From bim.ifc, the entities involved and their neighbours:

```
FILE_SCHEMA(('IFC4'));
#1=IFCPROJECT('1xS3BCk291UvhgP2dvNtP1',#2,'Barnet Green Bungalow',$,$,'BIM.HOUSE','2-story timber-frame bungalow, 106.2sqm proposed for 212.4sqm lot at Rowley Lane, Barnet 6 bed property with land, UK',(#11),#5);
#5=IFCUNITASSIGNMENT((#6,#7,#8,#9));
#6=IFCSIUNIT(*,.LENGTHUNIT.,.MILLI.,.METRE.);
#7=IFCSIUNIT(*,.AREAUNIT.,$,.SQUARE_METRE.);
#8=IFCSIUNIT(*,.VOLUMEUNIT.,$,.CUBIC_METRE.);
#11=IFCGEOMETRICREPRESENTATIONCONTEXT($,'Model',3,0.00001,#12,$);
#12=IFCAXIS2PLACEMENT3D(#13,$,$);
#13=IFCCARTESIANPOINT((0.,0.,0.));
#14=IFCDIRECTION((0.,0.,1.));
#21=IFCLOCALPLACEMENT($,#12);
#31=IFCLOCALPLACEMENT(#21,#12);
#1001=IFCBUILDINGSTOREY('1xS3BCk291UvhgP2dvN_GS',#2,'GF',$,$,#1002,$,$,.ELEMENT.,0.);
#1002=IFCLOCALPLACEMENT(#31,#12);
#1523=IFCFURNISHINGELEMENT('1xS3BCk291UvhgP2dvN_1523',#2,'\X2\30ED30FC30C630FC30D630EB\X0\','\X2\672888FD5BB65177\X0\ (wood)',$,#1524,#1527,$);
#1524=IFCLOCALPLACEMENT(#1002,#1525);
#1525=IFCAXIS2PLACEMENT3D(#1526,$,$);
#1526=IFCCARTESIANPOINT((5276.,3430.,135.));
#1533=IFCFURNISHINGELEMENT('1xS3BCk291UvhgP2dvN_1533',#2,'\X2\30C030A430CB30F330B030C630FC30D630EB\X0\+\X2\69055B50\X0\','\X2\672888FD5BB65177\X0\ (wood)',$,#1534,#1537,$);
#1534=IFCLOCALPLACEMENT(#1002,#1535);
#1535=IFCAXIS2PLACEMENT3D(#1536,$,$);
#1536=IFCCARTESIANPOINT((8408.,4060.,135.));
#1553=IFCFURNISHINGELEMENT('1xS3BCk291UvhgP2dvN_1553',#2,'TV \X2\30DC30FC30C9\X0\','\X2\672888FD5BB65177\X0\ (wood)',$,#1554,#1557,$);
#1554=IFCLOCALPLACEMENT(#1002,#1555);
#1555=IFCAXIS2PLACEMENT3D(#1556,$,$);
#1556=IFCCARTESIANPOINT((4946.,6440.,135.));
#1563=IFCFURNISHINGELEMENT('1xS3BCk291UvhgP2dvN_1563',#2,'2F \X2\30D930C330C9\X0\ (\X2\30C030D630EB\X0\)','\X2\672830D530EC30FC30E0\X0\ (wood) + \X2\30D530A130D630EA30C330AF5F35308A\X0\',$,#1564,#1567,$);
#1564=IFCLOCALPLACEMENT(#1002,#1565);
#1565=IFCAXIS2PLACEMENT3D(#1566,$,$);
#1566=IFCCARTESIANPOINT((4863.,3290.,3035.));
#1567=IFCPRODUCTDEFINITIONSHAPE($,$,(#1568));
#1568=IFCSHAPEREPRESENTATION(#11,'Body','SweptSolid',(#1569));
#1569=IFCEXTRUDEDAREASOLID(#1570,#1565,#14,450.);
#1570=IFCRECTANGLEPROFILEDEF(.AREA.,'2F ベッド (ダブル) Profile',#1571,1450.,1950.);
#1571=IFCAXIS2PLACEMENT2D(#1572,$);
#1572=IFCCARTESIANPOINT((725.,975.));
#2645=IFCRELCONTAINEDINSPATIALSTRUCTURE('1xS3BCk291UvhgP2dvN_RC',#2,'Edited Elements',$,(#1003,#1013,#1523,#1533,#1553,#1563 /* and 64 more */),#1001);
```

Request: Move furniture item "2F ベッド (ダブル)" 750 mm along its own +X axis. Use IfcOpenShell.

```python
import ifcopenshell
import ifcopenshell.api.geometry
import ifcopenshell.util.placement
import ifcopenshell.util.unit

model = ifcopenshell.open("bim.ifc")
unit_scale = ifcopenshell.util.unit.calculate_unit_scale(model)

item = model.by_guid("1xS3BCk291UvhgP2dvN_1563")
matrix = ifcopenshell.util.placement.get_local_placement(item.ObjectPlacement)
matrix[:3, 3] += matrix[:3, 0] * 0.75 / unit_scale
ifcopenshell.api.geometry.edit_object_placement(model, product=item, matrix=matrix, is_si=False)

print(ifcopenshell.util.placement.get_local_placement(item.ObjectPlacement).round(3) + 0.0)

model.write("bim_rev.ifc")
```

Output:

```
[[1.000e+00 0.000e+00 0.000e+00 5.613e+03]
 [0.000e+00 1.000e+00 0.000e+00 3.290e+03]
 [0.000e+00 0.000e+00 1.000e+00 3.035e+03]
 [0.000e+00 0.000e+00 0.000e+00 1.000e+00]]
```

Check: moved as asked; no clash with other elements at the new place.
